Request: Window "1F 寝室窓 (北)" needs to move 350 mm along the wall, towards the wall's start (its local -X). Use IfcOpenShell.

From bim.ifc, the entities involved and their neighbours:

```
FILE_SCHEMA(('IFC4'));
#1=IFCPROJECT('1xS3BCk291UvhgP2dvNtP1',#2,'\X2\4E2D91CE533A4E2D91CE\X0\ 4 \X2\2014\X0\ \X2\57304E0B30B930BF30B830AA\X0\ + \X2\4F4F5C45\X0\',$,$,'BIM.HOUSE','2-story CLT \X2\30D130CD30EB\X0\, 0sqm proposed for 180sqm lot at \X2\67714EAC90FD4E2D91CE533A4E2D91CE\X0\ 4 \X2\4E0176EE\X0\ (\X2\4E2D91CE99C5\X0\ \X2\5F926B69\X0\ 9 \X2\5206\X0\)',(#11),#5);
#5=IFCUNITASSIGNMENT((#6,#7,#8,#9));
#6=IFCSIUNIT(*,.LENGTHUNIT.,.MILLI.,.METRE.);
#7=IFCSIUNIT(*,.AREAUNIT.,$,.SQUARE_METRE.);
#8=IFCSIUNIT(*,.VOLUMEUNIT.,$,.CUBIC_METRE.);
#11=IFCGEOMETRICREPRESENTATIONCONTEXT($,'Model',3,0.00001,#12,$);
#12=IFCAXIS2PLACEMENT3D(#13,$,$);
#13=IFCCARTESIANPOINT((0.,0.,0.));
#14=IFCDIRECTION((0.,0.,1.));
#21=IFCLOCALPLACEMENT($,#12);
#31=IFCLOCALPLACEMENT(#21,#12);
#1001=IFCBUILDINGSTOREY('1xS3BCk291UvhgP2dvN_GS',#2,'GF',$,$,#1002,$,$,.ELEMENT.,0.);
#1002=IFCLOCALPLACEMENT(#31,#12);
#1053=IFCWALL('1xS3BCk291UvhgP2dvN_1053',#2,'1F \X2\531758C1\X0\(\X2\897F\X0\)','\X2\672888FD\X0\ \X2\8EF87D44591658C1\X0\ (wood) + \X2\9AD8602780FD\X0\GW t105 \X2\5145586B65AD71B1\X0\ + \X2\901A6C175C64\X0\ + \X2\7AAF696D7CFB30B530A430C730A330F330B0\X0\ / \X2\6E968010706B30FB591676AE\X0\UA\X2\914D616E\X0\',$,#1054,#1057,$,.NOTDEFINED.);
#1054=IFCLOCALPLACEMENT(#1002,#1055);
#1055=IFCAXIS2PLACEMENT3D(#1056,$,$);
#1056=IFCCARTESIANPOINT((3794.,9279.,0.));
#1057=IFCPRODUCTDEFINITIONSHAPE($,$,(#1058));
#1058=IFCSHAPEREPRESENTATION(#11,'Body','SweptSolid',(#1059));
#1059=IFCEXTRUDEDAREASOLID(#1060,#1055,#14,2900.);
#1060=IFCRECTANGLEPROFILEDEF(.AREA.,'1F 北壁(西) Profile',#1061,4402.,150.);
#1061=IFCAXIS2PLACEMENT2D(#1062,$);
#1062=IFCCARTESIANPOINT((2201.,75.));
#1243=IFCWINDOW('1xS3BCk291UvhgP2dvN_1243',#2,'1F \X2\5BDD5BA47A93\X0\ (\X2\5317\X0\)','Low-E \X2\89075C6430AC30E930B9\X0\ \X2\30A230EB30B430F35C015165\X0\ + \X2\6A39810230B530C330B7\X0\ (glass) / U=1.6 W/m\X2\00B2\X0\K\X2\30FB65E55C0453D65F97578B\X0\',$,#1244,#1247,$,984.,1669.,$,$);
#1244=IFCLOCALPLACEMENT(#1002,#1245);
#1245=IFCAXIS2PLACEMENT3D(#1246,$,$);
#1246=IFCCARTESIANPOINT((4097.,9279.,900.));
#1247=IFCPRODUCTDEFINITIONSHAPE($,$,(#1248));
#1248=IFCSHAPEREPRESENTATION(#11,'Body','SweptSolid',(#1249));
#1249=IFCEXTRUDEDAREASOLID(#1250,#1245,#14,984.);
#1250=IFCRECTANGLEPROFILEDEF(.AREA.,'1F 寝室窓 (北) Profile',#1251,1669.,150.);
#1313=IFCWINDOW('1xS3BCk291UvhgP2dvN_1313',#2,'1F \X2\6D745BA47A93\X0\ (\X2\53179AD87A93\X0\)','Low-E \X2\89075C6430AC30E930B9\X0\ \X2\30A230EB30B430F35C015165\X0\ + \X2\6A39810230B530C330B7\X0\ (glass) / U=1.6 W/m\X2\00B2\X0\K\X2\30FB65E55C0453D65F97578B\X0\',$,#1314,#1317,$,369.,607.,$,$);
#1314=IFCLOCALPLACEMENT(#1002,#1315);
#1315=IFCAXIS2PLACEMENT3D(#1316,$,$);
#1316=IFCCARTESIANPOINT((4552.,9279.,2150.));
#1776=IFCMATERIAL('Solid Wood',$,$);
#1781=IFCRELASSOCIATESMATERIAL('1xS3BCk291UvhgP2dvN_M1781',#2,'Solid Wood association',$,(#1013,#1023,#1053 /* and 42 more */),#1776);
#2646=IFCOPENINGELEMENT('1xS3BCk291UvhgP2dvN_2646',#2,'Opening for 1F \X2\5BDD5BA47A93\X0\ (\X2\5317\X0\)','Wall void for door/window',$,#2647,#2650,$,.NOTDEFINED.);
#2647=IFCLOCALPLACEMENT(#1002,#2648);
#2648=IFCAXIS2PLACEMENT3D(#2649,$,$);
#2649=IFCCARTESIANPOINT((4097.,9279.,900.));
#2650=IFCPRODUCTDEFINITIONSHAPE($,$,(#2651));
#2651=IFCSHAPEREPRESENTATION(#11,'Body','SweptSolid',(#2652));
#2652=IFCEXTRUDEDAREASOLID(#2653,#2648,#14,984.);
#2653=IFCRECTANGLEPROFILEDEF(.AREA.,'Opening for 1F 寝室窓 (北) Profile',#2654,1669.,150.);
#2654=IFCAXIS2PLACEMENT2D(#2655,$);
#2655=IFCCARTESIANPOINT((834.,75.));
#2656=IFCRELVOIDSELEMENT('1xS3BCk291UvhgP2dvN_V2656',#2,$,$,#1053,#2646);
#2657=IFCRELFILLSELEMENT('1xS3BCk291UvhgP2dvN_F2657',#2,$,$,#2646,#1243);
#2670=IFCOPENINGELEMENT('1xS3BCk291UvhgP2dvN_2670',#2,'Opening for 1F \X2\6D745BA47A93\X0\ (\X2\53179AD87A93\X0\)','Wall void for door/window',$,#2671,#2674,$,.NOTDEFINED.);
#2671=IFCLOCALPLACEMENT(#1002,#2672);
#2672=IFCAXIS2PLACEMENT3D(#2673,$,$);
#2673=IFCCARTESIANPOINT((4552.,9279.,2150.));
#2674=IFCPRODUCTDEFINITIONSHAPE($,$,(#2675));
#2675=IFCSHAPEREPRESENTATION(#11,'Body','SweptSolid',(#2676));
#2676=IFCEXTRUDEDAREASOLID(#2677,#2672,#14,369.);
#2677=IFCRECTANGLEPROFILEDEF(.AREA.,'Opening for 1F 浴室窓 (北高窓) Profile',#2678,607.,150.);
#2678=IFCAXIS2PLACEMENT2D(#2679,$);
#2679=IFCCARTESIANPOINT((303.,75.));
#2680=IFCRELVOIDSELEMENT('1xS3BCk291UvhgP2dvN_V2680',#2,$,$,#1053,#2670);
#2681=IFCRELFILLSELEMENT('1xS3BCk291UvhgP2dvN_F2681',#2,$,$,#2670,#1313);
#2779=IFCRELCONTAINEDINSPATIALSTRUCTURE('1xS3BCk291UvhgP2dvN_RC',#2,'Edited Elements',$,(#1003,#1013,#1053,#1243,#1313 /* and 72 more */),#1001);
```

```python
import ifcopenshell
import ifcopenshell.api.geometry
import ifcopenshell.util.placement

model = ifcopenshell.open("bim.ifc")

window = model.by_guid("1xS3BCk291UvhgP2dvN_1243")
opening = window.FillsVoids[0].RelatingOpeningElement
wall = opening.VoidsElements[0].RelatingBuildingElement

wall_matrix = ifcopenshell.util.placement.get_local_placement(wall.ObjectPlacement)
shift = wall_matrix[:3, 0] * -350.0
before = ifcopenshell.util.placement.get_local_placement(window.ObjectPlacement)[:3, 3].copy()

# The window is not placed relative to its opening, so move both.
for product in (opening, window):
    matrix = ifcopenshell.util.placement.get_local_placement(product.ObjectPlacement)
    matrix[:3, 3] += shift
    ifcopenshell.api.geometry.edit_object_placement(model, product=product, matrix=matrix, is_si=False)

after = ifcopenshell.util.placement.get_local_placement(window.ObjectPlacement)[:3, 3]
print("window moved by", (after - before).round(3) + 0.0)

model.write("bim-out.ifc")
```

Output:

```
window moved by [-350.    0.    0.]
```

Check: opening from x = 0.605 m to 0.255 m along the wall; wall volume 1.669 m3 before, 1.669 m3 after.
